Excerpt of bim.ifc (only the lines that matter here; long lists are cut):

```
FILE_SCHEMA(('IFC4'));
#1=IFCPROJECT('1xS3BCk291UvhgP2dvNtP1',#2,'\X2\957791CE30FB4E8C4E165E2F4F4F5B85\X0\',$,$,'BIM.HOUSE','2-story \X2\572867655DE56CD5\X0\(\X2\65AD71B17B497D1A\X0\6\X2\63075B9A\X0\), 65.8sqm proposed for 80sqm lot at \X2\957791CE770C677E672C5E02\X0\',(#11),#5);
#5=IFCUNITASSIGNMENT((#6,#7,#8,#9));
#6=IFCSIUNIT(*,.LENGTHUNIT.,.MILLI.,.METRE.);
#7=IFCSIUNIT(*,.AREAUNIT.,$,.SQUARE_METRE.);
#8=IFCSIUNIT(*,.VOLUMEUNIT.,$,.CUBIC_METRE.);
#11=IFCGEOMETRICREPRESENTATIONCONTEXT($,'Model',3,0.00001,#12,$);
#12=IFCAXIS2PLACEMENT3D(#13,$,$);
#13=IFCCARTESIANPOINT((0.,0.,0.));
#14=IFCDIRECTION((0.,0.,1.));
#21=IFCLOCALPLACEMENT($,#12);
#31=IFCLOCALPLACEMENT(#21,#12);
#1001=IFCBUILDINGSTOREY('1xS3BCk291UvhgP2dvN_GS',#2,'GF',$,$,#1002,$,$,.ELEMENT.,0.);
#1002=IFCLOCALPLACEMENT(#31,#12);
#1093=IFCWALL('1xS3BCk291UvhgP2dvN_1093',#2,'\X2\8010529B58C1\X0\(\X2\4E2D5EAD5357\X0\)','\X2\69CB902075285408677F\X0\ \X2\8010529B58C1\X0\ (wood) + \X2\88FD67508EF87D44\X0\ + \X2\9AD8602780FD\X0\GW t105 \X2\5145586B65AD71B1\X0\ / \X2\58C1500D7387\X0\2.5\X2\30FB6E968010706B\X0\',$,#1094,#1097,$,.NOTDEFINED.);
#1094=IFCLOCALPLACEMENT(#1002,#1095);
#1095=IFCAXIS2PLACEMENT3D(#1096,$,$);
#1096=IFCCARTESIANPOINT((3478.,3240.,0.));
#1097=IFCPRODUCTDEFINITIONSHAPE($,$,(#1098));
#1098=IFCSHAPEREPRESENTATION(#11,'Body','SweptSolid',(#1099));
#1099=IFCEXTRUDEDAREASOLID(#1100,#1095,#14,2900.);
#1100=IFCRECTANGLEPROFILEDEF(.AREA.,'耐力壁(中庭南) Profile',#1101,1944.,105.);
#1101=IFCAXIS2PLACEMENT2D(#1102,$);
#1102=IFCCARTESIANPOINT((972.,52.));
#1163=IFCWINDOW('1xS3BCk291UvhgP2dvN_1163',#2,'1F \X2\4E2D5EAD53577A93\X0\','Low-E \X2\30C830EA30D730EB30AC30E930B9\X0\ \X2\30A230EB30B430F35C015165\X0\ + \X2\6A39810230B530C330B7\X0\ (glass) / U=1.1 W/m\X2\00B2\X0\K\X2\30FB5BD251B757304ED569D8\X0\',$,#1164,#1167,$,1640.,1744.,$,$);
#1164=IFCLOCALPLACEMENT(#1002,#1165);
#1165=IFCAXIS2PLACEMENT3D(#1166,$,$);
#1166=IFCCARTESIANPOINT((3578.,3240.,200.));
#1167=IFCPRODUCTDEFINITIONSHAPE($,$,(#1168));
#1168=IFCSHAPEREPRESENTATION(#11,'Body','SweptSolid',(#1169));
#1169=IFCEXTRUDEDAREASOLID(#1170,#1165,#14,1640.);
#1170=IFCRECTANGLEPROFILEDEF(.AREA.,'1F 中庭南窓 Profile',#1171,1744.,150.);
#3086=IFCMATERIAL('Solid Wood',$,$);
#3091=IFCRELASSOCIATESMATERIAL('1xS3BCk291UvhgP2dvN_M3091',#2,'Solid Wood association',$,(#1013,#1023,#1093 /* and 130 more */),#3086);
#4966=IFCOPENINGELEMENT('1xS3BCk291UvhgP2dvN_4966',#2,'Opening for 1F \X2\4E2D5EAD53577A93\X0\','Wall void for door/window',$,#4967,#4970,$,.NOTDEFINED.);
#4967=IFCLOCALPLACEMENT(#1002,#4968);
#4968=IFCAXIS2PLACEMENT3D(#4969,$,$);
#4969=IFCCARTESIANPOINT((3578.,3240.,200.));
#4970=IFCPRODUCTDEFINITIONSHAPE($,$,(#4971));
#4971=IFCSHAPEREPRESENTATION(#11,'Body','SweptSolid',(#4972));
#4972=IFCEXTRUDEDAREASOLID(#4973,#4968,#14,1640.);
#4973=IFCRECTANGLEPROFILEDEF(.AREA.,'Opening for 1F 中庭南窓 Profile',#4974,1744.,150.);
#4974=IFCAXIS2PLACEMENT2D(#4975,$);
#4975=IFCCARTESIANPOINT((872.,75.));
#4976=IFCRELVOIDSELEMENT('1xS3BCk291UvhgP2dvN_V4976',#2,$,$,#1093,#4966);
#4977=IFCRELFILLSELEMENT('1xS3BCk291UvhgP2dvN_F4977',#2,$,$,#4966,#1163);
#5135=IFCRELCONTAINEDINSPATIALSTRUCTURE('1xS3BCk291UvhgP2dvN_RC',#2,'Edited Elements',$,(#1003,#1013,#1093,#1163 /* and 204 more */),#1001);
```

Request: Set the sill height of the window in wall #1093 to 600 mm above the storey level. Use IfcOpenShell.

```python
import numpy as np
import ifcopenshell
import ifcopenshell.api.geometry
import ifcopenshell.geom
import ifcopenshell.util.element
import ifcopenshell.util.placement
import ifcopenshell.util.shape
import ifcopenshell.util.unit

model = ifcopenshell.open("bim.ifc")
unit_scale = ifcopenshell.util.unit.calculate_unit_scale(model)

window = model.by_guid("1xS3BCk291UvhgP2dvN_1163")
opening = window.FillsVoids[0].RelatingOpeningElement
storey = ifcopenshell.util.element.get_container(window, ifc_class="IfcBuildingStorey")
level = ifcopenshell.util.placement.get_local_placement(storey.ObjectPlacement)[2, 3]

# The opening's origin need not be at the sill, so measure its lowest point.
shape = ifcopenshell.geom.create_shape(ifcopenshell.geom.settings(), opening)
bottom = ifcopenshell.util.shape.get_shape_bottom_elevation(shape, shape.geometry) / unit_scale
dz = level + 0.6 / unit_scale - bottom

shift = np.array([0.0, 0.0, dz])
# The window is not placed relative to its opening, so move both.
for product in (opening, window):
    matrix = ifcopenshell.util.placement.get_local_placement(product.ObjectPlacement)
    matrix[:3, 3] += shift
    ifcopenshell.api.geometry.edit_object_placement(model, product=product, matrix=matrix, is_si=False)

print(f"moved by {dz * unit_scale:+.3f} m")

model.write("bim-out.ifc")
```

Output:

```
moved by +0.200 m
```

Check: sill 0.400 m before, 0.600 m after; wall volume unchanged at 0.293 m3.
